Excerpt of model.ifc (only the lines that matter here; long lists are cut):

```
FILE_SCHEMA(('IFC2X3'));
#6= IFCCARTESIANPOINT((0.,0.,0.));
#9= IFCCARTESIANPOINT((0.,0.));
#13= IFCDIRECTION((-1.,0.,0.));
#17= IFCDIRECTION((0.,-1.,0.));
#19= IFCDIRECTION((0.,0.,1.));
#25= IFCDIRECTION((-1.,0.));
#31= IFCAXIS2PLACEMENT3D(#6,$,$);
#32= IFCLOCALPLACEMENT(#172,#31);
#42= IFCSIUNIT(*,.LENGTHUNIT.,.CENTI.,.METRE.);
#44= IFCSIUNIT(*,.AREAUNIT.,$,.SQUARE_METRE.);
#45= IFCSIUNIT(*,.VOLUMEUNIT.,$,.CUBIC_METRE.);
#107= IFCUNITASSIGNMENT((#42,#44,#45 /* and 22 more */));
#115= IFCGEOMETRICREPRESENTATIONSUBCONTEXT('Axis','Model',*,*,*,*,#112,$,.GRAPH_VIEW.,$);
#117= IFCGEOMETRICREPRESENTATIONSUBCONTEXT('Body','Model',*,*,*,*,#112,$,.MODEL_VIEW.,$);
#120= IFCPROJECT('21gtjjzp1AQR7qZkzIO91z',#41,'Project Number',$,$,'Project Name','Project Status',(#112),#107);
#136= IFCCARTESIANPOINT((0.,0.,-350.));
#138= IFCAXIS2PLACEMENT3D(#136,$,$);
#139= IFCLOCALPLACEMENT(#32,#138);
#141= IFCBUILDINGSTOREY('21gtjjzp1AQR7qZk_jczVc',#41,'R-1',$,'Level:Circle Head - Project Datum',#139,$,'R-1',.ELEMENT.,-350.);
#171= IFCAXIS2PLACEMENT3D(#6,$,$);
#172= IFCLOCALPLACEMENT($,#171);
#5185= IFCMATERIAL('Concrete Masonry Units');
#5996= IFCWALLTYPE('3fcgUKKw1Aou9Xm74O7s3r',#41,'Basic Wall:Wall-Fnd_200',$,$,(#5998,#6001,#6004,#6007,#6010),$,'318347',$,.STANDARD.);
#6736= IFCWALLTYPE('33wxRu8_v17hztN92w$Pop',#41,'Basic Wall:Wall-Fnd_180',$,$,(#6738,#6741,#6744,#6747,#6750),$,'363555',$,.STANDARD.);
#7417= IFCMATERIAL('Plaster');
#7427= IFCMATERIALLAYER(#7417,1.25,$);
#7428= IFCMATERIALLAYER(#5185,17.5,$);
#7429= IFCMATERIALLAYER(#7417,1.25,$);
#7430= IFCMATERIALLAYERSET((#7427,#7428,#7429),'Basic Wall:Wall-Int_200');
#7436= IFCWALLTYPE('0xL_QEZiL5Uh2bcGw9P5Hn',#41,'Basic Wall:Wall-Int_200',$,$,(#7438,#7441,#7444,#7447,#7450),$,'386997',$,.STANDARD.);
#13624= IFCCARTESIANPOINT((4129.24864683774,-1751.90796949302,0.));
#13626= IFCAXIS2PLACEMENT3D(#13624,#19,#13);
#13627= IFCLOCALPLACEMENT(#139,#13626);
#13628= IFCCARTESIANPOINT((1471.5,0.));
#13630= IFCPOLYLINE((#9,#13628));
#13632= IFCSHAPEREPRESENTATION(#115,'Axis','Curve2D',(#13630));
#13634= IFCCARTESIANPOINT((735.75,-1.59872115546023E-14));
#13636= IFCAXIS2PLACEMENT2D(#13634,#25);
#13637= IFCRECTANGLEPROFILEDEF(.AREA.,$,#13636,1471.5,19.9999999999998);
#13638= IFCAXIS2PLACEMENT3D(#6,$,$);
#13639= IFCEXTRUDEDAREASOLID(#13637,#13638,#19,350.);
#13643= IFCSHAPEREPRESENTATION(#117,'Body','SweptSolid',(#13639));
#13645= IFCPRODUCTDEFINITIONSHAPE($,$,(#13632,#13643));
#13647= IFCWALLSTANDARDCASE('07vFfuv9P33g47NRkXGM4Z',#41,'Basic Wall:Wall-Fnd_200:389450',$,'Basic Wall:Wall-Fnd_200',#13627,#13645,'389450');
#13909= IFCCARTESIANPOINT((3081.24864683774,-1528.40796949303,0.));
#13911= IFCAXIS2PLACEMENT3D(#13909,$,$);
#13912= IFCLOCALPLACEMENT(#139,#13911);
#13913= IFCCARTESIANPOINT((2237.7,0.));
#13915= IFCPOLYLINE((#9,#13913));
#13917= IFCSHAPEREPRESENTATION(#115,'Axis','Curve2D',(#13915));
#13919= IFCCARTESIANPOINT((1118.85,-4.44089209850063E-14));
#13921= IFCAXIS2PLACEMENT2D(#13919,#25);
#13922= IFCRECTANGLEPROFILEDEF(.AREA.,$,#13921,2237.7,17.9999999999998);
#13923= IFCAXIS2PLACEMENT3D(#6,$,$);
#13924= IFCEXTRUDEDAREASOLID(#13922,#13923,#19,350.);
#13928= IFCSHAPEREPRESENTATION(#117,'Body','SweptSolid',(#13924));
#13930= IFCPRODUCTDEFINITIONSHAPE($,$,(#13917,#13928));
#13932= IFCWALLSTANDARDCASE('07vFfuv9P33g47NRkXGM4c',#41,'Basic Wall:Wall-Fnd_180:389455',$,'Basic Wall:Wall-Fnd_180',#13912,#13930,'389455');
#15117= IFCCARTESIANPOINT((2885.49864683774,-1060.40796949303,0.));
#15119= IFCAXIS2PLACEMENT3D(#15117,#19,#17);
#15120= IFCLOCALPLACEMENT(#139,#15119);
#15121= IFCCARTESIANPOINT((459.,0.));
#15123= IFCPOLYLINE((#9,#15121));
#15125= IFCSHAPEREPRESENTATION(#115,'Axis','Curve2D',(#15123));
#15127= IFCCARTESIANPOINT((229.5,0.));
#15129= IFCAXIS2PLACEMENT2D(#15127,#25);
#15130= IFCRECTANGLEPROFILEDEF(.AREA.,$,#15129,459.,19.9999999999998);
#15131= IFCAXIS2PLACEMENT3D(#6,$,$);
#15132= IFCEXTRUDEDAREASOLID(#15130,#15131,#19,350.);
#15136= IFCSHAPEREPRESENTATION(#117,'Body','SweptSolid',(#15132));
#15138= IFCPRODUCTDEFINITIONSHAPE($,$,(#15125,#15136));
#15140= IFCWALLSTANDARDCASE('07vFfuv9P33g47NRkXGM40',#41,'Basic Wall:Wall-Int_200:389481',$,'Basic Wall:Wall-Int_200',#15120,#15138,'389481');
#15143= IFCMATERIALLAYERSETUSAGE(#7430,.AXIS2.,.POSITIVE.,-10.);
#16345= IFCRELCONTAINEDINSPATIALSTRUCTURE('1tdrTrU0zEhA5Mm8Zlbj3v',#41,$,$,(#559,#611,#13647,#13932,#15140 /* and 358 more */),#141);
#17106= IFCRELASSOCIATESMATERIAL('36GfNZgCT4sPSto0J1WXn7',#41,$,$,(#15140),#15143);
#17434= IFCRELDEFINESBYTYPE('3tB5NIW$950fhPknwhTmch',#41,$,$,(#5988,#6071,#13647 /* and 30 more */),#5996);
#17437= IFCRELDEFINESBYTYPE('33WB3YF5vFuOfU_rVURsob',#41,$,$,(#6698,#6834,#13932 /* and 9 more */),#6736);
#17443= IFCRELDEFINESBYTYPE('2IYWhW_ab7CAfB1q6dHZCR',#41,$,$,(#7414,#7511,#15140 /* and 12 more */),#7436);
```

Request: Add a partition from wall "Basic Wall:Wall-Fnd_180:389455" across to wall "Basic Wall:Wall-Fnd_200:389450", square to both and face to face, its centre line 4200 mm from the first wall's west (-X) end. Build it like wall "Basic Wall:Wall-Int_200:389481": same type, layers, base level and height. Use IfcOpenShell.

```python
import numpy as np
import ifcopenshell
import ifcopenshell.api.geometry
import ifcopenshell.api.material
import ifcopenshell.api.pset
import ifcopenshell.api.root
import ifcopenshell.api.spatial
import ifcopenshell.api.type
import ifcopenshell.geom
import ifcopenshell.util.element
import ifcopenshell.util.placement
import ifcopenshell.util.representation
import ifcopenshell.util.shape
import ifcopenshell.util.unit

model = ifcopenshell.open("model.ifc")
unit_scale = ifcopenshell.util.unit.calculate_unit_scale(model)
settings = ifcopenshell.geom.settings()
settings.set("use-world-coords", True)

start_wall = model.by_id(13932)
end_wall = model.by_guid("07vFfuv9P33g47NRkXGM4Z")
like = model.by_id(15140)
matrix = ifcopenshell.util.placement.get_local_placement(start_wall.ObjectPlacement)
matrix[:3, 3] *= unit_scale


def extent(element):
    """Bounding box in the first wall's axes, in metres."""
    shape = ifcopenshell.geom.create_shape(settings, element)
    points = (ifcopenshell.util.shape.get_vertices(shape.geometry) - matrix[:3, 3]) @ matrix[:3, :3]
    return points.min(axis=0), points.max(axis=0)


y_start = extent(start_wall)[0][1]
y_end = extent(end_wall)[1][1]
like_min, like_max = extent(like)
length, height = float(abs(y_end - y_start)), float(like_max[2] - like_min[2])
layer_set = ifcopenshell.util.element.get_material(like, should_skip_usage=True)
thickness = sum(layer.LayerThickness for layer in layer_set.MaterialLayers) * unit_scale

wall = ifcopenshell.api.root.create_entity(model, ifc_class="IfcWallStandardCase", name="New partition")
storey = ifcopenshell.util.element.get_container(like)
ifcopenshell.api.spatial.assign_container(model, products=[wall], relating_structure=storey)
ifcopenshell.api.type.assign_type(
    model, related_objects=[wall], relating_type=ifcopenshell.util.element.get_type(like), should_map_representations=False
)
rel = ifcopenshell.api.material.assign_material(
    model, products=[wall], type="IfcMaterialLayerSetUsage", material=layer_set
)
rel.RelatingMaterial.OffsetFromReferenceLine = -thickness / 2 / unit_scale
pset = ifcopenshell.api.pset.add_pset(model, product=wall, name="Pset_WallCommon")
ifcopenshell.api.pset.edit_pset(model, pset=pset, properties={"IsExternal": False, "LoadBearing": False})

# The axis runs down the middle of the wall.
axis = ifcopenshell.api.geometry.add_axis_representation(
    model, context=ifcopenshell.util.representation.get_context(model, "Model", "Axis"), axis=[(0.0, 0.0), (length, 0.0)]
)
body = ifcopenshell.api.geometry.add_wall_representation(
    model,
    context=ifcopenshell.util.representation.get_context(model, "Model", "Body", "MODEL_VIEW"),
    length=length,
    height=height,
    thickness=thickness,
    offset=-thickness / 2,
)
for representation in (axis, body):
    ifcopenshell.api.geometry.assign_representation(model, product=wall, representation=representation)

placement = matrix @ ifcopenshell.util.placement.rotation(-90, "Z")
placement[:, 3] = matrix @ np.array([extent(start_wall)[0][0] + 4.2, y_start, like_min[2], 1.0])
ifcopenshell.api.geometry.edit_object_placement(model, product=wall, matrix=placement)

print(f"partition {length:.3f} m long, {height:.3f} m high, {thickness:.3f} m thick")

model.write("model-out.ifc")
```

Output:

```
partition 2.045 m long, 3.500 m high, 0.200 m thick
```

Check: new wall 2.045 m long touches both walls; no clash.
